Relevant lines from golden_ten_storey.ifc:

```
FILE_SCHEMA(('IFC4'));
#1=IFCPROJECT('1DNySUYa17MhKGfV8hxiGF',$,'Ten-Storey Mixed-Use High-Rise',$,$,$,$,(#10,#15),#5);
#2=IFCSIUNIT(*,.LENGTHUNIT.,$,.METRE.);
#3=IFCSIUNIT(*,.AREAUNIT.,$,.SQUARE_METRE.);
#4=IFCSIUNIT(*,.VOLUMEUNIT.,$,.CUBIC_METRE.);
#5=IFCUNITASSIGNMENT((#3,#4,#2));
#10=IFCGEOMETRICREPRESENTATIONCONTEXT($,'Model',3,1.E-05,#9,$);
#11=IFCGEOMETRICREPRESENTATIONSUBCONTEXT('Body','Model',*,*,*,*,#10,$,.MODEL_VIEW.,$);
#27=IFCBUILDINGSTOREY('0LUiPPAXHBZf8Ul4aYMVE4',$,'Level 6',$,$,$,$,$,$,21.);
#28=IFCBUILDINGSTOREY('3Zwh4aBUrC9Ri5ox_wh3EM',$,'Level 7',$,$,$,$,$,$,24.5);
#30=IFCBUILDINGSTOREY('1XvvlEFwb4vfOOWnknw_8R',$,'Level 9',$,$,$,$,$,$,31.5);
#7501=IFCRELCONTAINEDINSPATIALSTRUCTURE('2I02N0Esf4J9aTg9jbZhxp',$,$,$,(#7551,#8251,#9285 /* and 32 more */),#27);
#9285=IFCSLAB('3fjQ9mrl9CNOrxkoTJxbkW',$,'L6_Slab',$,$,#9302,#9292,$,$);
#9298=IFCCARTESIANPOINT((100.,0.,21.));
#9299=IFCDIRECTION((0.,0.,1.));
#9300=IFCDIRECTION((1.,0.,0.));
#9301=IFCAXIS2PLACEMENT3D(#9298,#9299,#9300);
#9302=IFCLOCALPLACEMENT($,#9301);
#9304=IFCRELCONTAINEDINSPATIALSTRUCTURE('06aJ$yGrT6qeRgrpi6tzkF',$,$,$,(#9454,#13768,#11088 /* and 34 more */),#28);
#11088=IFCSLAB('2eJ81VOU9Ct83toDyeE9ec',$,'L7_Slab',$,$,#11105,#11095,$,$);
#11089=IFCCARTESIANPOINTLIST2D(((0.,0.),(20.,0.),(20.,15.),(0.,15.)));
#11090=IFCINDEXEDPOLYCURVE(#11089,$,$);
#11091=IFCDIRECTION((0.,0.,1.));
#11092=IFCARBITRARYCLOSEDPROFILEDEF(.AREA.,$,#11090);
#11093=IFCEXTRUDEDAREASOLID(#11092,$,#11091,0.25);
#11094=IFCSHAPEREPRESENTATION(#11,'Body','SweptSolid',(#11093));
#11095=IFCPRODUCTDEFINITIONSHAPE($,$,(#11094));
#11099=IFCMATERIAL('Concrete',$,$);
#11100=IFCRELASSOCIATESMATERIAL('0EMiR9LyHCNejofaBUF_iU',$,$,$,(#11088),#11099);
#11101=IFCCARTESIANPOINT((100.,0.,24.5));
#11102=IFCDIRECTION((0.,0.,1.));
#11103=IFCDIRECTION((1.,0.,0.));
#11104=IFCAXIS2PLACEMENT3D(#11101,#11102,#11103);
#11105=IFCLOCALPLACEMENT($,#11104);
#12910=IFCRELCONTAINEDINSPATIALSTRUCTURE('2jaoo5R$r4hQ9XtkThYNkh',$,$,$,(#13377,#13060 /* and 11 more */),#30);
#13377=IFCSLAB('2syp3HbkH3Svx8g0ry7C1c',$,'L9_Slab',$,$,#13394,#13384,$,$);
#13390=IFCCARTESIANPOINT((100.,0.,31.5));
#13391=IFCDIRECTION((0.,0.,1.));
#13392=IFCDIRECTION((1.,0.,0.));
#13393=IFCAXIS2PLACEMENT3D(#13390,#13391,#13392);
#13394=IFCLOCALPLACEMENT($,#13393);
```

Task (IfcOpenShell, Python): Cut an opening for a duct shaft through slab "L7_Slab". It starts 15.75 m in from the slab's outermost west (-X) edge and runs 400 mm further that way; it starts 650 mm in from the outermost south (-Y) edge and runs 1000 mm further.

```python
import numpy as np
import ifcopenshell
import ifcopenshell.api.feature
import ifcopenshell.api.geometry
import ifcopenshell.api.root
import ifcopenshell.geom
import ifcopenshell.util.placement
import ifcopenshell.util.representation
import ifcopenshell.util.shape
import ifcopenshell.util.unit

model = ifcopenshell.open("golden_ten_storey.ifc")
unit_scale = ifcopenshell.util.unit.calculate_unit_scale(model)
settings = ifcopenshell.geom.settings()


def volume(element):
    """Net volume in cubic metres, openings subtracted."""
    shape = ifcopenshell.geom.create_shape(settings, element)
    return ifcopenshell.util.shape.get_volume(shape.geometry)


slab = model.by_guid("2eJ81VOU9Ct83toDyeE9ec")
before = volume(slab)

# Extent in the slab's own axes, in metres. The edges named are its -X and -Y sides.
slab_shape = ifcopenshell.geom.create_shape(settings, slab)
vertices = ifcopenshell.util.shape.get_vertices(slab_shape.geometry)
x_min, y_min, bottom = vertices.min(axis=0)
top = vertices[:, 2].max()

opening = ifcopenshell.api.root.create_entity(model, ifc_class="IfcOpeningElement", name="Duct shaft opening", predefined_type="OPENING")
context = ifcopenshell.util.representation.get_context(model, "Model", "Body", "MODEL_VIEW")
width, depth = 0.4, 1
outline = [(0.0, 0.0), (width, 0.0), (width, depth), (0.0, depth), (0.0, 0.0)]
# Overshoot both faces by 50 mm so the cut is clean.
shape = ifcopenshell.api.geometry.add_slab_representation(
    model, context=context, depth=top - bottom + 0.1, polyline=outline
)
ifcopenshell.api.geometry.assign_representation(model, product=opening, representation=shape)

matrix = ifcopenshell.util.placement.get_local_placement(slab.ObjectPlacement)
matrix[:, 3] = matrix @ np.append(np.array([x_min + 15.75, y_min + 0.65, bottom - 0.05]) / unit_scale, 1.0)
ifcopenshell.api.geometry.edit_object_placement(model, product=opening, matrix=matrix, is_si=False)
ifcopenshell.api.feature.add_feature(model, feature=opening, element=slab)

after = volume(slab)

print(f"slab volume {before:.3f} -> {after:.3f} m3")

model.write("golden_ten_storey_rev.ifc")
```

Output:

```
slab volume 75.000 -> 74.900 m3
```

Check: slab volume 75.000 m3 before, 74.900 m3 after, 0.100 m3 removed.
